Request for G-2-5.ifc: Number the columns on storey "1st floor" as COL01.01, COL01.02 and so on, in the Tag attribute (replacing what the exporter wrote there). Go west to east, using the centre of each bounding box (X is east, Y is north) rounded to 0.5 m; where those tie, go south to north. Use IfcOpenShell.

First a look at what the model holds.

```python
import ifcopenshell
import ifcopenshell.util.element
import ifcopenshell.util.placement

model = ifcopenshell.open("G-2-5.ifc")
print(model.schema)
storey = next(s for s in model.by_type("IfcBuildingStorey") if s.Name == "1st floor")
columns = [e for e in ifcopenshell.util.element.get_decomposition(storey) if e.is_a("IfcColumn")]
for e in sorted(columns, key=lambda e: e.id()):
    origin = ifcopenshell.util.placement.get_local_placement(e.ObjectPlacement)[:3, 3]
    print(e.id(), e.Tag, e.Name, origin.round(2) + 0.0, sep=" | ")
```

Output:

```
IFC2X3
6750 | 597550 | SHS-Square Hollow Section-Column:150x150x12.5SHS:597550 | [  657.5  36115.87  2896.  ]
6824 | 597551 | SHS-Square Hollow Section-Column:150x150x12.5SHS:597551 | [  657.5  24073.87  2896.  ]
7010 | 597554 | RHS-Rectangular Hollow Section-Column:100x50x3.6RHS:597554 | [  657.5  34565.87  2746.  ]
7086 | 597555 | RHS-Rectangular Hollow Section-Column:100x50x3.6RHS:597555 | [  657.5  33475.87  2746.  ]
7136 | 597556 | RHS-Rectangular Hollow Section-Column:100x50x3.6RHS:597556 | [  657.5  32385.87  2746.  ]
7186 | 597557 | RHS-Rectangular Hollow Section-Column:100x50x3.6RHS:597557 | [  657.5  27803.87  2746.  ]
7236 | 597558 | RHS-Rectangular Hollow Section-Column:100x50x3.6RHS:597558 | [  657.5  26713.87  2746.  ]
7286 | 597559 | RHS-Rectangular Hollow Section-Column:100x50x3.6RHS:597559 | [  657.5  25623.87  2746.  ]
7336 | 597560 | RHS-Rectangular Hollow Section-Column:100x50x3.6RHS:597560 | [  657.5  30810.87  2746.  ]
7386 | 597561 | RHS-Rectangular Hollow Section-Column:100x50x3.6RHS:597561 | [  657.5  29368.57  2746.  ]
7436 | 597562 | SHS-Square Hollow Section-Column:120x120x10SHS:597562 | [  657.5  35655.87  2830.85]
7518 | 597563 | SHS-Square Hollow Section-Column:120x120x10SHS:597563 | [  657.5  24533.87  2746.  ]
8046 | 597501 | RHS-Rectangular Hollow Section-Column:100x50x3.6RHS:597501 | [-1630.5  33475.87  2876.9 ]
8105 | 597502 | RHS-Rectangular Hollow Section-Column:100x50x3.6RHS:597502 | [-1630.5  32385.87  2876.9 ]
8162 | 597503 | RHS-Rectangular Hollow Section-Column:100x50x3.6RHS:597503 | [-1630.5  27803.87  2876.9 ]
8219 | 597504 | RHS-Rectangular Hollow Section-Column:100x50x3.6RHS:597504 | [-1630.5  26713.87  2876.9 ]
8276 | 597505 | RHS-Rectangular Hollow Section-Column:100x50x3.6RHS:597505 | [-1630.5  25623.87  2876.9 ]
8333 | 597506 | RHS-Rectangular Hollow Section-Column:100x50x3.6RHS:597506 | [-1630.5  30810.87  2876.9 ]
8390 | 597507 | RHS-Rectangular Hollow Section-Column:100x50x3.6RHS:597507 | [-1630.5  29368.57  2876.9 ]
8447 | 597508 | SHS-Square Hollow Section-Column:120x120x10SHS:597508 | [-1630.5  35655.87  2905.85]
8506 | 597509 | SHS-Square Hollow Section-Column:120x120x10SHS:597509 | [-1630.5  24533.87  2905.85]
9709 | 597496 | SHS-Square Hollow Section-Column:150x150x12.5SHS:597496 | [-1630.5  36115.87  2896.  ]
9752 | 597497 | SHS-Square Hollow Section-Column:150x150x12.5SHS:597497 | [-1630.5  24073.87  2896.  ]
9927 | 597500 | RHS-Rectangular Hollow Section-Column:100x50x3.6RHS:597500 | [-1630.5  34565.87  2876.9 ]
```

```python
import ifcopenshell
import ifcopenshell.geom
import ifcopenshell.util.element
import ifcopenshell.util.shape

model = ifcopenshell.open("G-2-5.ifc")
settings = ifcopenshell.geom.settings()
settings.set("use-world-coords", True)


def centre(element):
    shape = ifcopenshell.geom.create_shape(settings, element)
    return ifcopenshell.util.shape.get_bbox_centroid(shape.geometry)


storey = next(s for s in model.by_type("IfcBuildingStorey") if s.Name == "1st floor")
columns = [e for e in ifcopenshell.util.element.get_decomposition(storey) if e.is_a("IfcColumn")]

# Insertion points can sit at a corner or the storey origin, so sort by the geometry (in metres).
centres = {e: centre(e) for e in columns}
columns.sort(key=lambda e: (round(centres[e][0] / 0.5), centres[e][1]))

for i, e in enumerate(columns, start=1):
    number = f"COL01.{i:02d}"
    e.Tag = number
    print(e.id(), number)

model.write("G-2-5_v2.ifc")
```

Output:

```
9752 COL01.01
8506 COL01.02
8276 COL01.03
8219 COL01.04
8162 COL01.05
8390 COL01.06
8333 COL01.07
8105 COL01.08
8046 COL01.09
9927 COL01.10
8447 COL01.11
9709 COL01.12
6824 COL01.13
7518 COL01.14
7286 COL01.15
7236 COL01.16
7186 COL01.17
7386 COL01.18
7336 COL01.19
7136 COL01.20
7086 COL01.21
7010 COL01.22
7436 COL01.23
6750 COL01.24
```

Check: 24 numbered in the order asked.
